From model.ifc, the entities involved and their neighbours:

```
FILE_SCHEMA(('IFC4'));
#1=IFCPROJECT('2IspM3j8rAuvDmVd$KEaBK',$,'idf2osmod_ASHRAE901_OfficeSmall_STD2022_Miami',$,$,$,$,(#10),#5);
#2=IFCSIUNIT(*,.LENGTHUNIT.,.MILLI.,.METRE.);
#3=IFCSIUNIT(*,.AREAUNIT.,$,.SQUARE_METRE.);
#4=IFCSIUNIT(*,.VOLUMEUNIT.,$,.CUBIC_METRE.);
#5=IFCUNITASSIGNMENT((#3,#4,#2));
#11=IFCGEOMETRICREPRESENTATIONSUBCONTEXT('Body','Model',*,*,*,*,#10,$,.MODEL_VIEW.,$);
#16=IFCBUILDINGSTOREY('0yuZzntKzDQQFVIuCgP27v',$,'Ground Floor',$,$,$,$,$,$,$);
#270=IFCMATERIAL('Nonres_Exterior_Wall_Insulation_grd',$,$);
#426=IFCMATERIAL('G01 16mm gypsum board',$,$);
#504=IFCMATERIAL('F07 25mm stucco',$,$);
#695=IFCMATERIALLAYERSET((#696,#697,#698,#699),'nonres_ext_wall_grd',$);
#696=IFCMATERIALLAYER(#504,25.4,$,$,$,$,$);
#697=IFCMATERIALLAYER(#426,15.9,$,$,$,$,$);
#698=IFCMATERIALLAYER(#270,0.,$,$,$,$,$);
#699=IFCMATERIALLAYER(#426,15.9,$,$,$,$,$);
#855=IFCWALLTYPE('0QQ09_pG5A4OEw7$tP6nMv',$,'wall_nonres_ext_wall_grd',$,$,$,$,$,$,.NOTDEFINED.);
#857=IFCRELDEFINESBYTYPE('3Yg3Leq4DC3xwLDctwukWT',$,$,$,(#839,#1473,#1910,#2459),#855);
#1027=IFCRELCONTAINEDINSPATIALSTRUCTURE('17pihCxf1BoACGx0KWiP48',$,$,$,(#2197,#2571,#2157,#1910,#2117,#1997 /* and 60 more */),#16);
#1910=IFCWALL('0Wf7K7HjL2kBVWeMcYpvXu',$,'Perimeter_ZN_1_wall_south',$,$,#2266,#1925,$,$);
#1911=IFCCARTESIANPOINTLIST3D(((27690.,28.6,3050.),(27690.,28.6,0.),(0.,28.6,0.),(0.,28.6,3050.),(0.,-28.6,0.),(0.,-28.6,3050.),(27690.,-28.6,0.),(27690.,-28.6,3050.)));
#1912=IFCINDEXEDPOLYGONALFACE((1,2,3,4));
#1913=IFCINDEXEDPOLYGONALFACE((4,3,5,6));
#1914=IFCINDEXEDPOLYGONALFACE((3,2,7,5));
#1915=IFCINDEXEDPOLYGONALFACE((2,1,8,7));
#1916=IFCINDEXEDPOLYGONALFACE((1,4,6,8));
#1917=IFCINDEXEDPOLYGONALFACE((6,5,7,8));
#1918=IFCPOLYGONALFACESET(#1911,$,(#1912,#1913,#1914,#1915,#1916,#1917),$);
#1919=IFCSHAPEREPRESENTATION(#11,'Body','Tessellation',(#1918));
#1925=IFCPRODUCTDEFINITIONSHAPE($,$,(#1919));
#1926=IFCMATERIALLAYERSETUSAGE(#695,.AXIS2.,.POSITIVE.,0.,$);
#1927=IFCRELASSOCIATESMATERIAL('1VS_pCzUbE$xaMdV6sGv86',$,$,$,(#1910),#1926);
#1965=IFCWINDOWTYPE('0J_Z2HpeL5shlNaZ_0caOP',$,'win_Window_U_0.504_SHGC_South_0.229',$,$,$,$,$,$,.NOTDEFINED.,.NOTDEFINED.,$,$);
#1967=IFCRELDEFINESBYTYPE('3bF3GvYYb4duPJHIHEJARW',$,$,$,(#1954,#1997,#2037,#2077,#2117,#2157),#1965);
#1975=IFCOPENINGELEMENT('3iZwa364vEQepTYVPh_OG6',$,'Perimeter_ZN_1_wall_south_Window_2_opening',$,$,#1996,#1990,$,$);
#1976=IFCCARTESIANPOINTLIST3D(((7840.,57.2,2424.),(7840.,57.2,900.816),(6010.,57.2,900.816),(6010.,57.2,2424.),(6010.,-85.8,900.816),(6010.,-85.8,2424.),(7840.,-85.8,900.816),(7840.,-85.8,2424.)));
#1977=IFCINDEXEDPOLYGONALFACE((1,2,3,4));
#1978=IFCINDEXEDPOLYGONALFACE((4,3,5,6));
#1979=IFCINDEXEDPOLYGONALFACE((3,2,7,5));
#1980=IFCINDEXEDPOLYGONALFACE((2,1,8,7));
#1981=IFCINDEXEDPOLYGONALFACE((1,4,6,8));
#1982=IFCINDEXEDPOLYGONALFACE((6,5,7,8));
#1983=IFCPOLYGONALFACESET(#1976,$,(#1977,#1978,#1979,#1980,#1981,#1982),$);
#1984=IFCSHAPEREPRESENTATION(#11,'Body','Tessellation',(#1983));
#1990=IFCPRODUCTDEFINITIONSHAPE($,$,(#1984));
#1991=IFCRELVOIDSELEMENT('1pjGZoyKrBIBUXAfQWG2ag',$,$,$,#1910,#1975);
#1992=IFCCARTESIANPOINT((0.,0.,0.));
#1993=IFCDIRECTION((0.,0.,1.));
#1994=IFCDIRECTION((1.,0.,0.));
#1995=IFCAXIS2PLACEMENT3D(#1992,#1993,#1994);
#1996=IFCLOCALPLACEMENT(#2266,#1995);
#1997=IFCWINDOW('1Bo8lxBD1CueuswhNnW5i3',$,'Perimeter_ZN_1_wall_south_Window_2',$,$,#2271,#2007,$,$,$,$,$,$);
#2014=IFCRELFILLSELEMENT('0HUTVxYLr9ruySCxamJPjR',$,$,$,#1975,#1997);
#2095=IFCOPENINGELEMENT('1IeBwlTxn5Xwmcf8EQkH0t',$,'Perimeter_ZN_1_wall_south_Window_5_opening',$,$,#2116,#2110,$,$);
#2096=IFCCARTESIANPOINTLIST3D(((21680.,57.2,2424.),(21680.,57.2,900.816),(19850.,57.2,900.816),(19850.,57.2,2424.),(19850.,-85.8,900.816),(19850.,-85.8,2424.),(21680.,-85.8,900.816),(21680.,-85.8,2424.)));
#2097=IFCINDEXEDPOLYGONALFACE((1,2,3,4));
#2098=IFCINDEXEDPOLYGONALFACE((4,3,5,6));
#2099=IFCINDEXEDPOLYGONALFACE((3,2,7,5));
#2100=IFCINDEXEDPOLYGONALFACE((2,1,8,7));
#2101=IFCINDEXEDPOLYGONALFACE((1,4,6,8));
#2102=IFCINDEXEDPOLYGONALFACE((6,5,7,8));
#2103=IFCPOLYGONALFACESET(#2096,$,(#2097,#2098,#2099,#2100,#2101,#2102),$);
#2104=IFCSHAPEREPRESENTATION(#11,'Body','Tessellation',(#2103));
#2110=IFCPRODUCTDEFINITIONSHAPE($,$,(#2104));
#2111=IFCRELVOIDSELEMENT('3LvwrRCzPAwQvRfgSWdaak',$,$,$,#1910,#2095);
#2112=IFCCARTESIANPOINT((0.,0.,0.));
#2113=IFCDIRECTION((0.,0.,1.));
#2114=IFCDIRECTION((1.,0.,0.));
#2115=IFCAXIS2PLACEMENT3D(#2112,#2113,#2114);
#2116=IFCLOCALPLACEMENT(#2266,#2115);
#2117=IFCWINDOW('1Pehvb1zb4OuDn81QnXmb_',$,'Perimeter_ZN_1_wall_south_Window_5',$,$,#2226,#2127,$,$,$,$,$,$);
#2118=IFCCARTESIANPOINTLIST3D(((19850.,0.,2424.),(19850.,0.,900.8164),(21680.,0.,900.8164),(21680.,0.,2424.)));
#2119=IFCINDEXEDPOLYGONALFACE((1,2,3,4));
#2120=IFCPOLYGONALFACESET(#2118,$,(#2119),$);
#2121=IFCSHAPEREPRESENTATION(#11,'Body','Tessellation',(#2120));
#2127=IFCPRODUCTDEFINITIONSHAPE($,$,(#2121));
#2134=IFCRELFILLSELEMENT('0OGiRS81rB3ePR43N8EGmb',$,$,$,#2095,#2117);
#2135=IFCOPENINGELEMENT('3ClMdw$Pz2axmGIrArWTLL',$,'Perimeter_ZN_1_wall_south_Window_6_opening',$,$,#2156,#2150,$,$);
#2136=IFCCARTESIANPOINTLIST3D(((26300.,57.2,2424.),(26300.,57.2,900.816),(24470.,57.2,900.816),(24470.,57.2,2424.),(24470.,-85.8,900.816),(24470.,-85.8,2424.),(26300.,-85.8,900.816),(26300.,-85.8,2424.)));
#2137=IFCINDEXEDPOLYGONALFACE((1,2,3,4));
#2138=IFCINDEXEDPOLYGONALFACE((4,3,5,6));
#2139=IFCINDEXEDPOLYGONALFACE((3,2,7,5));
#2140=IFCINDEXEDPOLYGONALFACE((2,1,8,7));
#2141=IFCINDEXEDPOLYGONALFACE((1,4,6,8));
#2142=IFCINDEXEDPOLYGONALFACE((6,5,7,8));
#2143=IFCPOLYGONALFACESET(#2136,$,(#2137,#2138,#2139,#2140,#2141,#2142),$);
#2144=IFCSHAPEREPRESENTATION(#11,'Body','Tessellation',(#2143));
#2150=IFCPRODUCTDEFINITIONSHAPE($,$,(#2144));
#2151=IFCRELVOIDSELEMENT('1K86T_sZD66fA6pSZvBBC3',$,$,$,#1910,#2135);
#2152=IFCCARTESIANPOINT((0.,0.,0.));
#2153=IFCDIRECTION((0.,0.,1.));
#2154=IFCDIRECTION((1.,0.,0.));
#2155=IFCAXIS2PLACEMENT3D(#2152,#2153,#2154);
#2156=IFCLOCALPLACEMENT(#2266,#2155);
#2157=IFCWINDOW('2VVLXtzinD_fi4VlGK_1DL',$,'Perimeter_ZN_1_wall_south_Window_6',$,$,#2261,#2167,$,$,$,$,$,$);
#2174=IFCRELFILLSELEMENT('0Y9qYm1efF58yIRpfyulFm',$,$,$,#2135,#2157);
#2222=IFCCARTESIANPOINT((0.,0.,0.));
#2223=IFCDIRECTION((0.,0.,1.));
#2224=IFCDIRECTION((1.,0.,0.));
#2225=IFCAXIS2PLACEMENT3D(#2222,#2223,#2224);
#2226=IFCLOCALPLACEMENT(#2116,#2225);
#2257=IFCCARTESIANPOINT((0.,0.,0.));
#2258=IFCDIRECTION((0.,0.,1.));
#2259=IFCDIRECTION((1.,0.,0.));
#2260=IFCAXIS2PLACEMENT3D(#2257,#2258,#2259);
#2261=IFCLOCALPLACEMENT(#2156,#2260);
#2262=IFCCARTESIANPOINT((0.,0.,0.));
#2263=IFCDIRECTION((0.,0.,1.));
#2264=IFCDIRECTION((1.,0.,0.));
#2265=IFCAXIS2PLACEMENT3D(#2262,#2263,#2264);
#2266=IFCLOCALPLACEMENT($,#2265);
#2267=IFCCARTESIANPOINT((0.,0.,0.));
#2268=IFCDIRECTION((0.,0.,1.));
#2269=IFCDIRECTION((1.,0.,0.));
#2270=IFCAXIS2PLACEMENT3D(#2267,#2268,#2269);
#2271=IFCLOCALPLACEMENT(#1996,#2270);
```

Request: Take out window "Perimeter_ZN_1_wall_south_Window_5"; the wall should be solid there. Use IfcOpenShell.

```python
import ifcopenshell
import ifcopenshell.api.feature
import ifcopenshell.api.root
import ifcopenshell.geom
import ifcopenshell.util.shape

model = ifcopenshell.open("model.ifc")
settings = ifcopenshell.geom.settings()


def volume(element):
    """Net volume in cubic metres, openings subtracted."""
    shape = ifcopenshell.geom.create_shape(settings, element)
    return ifcopenshell.util.shape.get_volume(shape.geometry)


window = model.by_id(2117)
opening = window.FillsVoids[0].RelatingOpeningElement
wall = opening.VoidsElements[0].RelatingBuildingElement
before = volume(wall)

ifcopenshell.api.root.remove_product(model, product=window)
ifcopenshell.api.feature.remove_feature(model, feature=opening)

after = volume(wall)

print(f"wall volume {before:.3f} -> {after:.3f} m3")

model.write("model_v2.ifc")
```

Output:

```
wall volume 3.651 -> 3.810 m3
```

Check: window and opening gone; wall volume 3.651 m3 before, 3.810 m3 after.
